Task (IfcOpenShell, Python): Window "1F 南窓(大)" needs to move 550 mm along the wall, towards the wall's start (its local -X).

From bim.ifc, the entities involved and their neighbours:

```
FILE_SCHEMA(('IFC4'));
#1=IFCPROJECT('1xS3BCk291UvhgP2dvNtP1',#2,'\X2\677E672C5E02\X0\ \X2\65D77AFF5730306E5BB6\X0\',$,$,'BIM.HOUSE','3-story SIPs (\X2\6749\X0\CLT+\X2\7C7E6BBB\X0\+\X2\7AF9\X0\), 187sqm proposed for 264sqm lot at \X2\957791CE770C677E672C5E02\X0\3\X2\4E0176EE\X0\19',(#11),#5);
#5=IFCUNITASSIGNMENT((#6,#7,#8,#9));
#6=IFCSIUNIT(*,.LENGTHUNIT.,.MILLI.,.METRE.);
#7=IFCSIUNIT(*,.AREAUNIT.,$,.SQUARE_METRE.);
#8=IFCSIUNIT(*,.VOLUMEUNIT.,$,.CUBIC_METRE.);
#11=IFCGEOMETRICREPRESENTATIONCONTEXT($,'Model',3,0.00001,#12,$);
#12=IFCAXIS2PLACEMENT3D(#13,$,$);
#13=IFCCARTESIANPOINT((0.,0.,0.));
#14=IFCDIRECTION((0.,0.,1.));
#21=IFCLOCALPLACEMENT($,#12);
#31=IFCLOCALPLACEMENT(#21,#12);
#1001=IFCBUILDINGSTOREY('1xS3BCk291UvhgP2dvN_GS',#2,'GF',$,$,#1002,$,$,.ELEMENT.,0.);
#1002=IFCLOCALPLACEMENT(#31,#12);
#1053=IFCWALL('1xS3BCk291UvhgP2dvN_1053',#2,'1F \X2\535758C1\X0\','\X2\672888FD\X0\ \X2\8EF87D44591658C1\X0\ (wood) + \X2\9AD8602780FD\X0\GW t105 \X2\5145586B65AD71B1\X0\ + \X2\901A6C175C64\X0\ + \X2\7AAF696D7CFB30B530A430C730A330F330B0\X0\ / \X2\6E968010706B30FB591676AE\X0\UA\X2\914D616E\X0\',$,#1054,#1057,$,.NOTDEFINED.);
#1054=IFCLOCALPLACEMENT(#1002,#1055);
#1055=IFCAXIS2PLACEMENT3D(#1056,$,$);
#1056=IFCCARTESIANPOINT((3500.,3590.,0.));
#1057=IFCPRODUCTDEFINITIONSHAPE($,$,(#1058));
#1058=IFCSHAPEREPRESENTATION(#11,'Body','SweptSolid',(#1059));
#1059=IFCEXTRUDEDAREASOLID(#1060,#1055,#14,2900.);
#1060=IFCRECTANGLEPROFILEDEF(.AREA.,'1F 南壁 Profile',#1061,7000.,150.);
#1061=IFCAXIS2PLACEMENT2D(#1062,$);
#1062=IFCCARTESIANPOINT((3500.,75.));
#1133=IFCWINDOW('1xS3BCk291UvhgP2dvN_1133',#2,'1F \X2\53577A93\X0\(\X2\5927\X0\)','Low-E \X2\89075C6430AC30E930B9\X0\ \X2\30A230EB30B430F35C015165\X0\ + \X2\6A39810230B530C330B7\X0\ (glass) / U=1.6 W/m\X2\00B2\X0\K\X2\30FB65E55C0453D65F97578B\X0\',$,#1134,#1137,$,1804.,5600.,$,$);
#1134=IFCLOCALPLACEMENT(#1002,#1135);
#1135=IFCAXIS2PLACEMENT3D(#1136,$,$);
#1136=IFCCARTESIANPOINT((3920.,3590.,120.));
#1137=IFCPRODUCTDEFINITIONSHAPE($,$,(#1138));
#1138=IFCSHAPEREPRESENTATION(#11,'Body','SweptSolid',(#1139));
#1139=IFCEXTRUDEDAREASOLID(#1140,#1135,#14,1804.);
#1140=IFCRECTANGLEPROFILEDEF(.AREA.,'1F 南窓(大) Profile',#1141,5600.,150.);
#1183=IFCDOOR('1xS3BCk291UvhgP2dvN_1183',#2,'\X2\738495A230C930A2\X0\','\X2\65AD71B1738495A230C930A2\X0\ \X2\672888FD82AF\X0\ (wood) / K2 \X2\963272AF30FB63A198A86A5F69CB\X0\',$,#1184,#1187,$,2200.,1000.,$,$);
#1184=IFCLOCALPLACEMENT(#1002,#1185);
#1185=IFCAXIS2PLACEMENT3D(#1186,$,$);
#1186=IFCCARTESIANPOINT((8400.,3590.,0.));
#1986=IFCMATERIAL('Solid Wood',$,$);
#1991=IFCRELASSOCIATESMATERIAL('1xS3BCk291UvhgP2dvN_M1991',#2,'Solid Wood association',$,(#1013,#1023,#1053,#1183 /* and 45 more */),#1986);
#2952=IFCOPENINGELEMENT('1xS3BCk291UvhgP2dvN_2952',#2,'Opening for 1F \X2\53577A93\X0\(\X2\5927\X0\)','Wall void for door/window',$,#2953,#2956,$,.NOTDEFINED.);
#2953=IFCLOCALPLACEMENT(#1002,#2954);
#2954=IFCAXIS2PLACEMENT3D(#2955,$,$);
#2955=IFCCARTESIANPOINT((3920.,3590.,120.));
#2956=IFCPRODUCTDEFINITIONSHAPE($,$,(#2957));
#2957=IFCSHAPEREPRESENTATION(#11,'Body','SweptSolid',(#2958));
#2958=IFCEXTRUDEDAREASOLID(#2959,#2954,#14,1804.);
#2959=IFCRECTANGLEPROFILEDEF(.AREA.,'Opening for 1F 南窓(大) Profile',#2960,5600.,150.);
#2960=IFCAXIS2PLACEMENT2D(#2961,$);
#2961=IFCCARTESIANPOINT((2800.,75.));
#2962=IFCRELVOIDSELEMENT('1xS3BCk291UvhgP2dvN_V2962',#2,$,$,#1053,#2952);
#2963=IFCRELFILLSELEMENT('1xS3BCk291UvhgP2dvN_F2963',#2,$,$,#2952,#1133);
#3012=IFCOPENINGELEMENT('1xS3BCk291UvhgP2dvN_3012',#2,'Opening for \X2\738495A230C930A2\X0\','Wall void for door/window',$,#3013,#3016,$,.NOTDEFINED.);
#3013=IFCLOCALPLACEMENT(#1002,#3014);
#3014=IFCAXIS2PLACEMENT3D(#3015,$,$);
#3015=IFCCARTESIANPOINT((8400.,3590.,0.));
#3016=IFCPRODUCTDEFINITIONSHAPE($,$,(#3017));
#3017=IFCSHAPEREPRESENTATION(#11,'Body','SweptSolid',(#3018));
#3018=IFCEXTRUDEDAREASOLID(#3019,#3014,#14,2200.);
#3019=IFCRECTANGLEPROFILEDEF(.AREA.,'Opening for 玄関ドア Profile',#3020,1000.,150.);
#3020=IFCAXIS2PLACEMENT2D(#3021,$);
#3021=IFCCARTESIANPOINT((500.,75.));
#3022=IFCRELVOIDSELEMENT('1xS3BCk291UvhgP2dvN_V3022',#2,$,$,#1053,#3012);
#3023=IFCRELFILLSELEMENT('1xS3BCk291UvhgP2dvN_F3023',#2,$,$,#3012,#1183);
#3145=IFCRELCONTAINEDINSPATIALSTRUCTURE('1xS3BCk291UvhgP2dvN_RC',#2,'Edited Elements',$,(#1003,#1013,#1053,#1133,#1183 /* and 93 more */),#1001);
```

```python
import ifcopenshell
import ifcopenshell.api.geometry
import ifcopenshell.util.placement

model = ifcopenshell.open("bim.ifc")

window = model.by_guid("1xS3BCk291UvhgP2dvN_1133")
opening = window.FillsVoids[0].RelatingOpeningElement
wall = opening.VoidsElements[0].RelatingBuildingElement

wall_matrix = ifcopenshell.util.placement.get_local_placement(wall.ObjectPlacement)
shift = wall_matrix[:3, 0] * -550.0
before = ifcopenshell.util.placement.get_local_placement(window.ObjectPlacement)[:3, 3].copy()

# The window is not placed relative to its opening, so move both.
for product in (opening, window):
    matrix = ifcopenshell.util.placement.get_local_placement(product.ObjectPlacement)
    matrix[:3, 3] += shift
    ifcopenshell.api.geometry.edit_object_placement(model, product=product, matrix=matrix, is_si=False)

after = ifcopenshell.util.placement.get_local_placement(window.ObjectPlacement)[:3, 3]
print("window moved by", (after - before).round(3) + 0.0)

model.write("bim_updated.ifc")
```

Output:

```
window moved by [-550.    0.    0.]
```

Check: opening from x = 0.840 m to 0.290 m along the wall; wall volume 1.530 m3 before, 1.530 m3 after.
